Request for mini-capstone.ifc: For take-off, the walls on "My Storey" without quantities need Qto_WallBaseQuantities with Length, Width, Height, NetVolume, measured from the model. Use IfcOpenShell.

First a look at what the model holds.

```python
import ifcopenshell
import ifcopenshell.util.element
import ifcopenshell.util.unit

model = ifcopenshell.open("mini-capstone.ifc")
print(model.schema)
for unit_type in ("LENGTHUNIT", "AREAUNIT", "VOLUMEUNIT"):
    print(unit_type, ifcopenshell.util.unit.calculate_unit_scale(model, unit_type))
storey = next(s for s in model.by_type("IfcBuildingStorey") if s.Name == "My Storey")
walls = [e for e in ifcopenshell.util.element.get_decomposition(storey) if e.is_a("IfcWall")]
for e in sorted(walls, key=lambda e: e.id()):
    print(e.id(), e.is_a(), e.Name, list(ifcopenshell.util.element.get_psets(e, qtos_only=True)), sep=" | ")
```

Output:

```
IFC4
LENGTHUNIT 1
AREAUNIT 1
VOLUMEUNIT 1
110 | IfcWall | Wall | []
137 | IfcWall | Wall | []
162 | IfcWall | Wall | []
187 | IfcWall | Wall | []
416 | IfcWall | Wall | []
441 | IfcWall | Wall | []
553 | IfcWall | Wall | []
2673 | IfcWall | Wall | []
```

```python
import ifcopenshell
import ifcopenshell.api.pset
import ifcopenshell.geom
import ifcopenshell.util.element
import ifcopenshell.util.shape
import ifcopenshell.util.unit

model = ifcopenshell.open("mini-capstone.ifc")
unit_scale = ifcopenshell.util.unit.calculate_unit_scale(model)
volume_scale = ifcopenshell.util.unit.calculate_unit_scale(model, "VOLUMEUNIT")
settings = ifcopenshell.geom.settings()

storey = next(s for s in model.by_type("IfcBuildingStorey") if s.Name == "My Storey")
walls = [e for e in ifcopenshell.util.element.get_decomposition(storey) if e.is_a("IfcWall")]

for e in sorted(walls, key=lambda e: e.id()):
    if ifcopenshell.util.element.get_psets(e, qtos_only=True, should_inherit=False):
        continue
    # Geometry comes back in metres, in the element's own axes.
    shape = ifcopenshell.geom.create_shape(settings, e)
    values = {
        "Length": ifcopenshell.util.shape.get_x(shape.geometry) / unit_scale,
        "Width": ifcopenshell.util.shape.get_y(shape.geometry) / unit_scale,
        "Height": ifcopenshell.util.shape.get_z(shape.geometry) / unit_scale,
        "NetVolume": ifcopenshell.util.shape.get_volume(shape.geometry) / volume_scale,
    }
    qto = ifcopenshell.api.pset.add_qto(model, product=e, name="Qto_WallBaseQuantities")
    ifcopenshell.api.pset.edit_qto(model, qto=qto, properties=values)
    print(e.id(), {k: round(v, 3) for k, v in values.items()})

model.write("mini-capstone_edited.ifc")
```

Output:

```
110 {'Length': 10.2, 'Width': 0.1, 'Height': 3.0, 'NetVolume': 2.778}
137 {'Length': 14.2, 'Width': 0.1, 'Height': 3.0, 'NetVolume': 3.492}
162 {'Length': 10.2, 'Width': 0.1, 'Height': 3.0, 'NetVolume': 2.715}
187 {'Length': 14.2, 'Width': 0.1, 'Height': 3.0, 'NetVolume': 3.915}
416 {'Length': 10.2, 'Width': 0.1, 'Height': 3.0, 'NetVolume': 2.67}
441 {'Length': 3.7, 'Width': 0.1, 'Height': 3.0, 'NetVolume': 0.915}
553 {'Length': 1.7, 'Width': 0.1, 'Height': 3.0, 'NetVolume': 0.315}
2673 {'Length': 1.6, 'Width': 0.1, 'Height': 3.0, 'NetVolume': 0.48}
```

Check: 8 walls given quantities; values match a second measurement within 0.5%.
